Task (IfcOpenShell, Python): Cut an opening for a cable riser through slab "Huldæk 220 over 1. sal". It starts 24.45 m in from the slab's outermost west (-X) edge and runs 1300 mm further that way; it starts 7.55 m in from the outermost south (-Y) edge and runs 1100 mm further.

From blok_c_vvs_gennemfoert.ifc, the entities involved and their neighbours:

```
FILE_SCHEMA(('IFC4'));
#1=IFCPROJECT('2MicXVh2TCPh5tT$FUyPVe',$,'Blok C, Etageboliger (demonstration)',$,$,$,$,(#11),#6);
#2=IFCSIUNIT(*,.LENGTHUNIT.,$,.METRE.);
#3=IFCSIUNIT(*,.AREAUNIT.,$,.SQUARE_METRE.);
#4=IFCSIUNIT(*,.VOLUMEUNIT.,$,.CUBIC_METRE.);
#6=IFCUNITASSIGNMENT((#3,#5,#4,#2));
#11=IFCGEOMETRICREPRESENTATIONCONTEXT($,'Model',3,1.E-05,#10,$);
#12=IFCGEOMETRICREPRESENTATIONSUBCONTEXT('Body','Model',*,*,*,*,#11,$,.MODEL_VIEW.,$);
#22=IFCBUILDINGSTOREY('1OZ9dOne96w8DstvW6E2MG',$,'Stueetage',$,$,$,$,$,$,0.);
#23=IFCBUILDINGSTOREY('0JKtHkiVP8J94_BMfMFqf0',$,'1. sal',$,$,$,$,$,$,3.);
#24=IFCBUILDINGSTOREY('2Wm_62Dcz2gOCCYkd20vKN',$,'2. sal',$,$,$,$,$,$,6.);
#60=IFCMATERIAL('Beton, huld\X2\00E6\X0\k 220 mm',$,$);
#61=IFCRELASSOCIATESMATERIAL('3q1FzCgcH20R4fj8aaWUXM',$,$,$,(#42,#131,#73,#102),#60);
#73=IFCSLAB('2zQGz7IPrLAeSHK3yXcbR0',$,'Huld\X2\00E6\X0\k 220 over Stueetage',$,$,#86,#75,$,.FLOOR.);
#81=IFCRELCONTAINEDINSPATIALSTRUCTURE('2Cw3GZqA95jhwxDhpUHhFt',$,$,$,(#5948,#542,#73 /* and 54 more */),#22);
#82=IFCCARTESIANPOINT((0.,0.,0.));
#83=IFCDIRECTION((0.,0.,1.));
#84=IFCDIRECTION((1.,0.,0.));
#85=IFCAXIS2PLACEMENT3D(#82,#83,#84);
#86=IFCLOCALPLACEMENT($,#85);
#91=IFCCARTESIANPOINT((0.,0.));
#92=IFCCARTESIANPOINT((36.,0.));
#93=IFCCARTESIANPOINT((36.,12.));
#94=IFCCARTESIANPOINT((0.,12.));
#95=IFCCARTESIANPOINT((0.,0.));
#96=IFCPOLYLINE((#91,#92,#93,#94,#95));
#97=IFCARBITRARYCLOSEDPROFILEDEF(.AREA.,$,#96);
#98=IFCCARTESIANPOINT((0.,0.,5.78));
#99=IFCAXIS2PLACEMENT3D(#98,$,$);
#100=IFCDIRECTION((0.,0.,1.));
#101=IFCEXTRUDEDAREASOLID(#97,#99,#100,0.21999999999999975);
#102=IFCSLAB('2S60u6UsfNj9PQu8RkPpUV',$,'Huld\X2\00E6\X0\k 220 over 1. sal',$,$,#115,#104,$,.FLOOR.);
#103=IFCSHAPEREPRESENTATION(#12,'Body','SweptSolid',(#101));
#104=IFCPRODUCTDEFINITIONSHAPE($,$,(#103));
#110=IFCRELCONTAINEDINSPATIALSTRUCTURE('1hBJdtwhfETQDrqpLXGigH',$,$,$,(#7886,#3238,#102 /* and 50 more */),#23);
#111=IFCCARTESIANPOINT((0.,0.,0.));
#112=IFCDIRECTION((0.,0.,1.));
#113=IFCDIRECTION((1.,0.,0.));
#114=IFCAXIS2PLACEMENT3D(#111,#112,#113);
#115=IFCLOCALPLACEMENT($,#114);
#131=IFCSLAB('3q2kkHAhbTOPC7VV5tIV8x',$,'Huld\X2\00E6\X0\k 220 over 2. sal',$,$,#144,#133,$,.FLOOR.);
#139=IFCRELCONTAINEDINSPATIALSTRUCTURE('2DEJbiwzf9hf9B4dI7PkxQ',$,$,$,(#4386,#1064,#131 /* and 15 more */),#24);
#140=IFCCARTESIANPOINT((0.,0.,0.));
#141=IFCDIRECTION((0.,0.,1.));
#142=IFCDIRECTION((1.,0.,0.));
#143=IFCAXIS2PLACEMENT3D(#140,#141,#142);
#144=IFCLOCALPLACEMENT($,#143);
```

```python
import numpy as np
import ifcopenshell
import ifcopenshell.api.feature
import ifcopenshell.api.geometry
import ifcopenshell.api.root
import ifcopenshell.geom
import ifcopenshell.util.placement
import ifcopenshell.util.representation
import ifcopenshell.util.shape
import ifcopenshell.util.unit

model = ifcopenshell.open("blok_c_vvs_gennemfoert.ifc")
unit_scale = ifcopenshell.util.unit.calculate_unit_scale(model)
settings = ifcopenshell.geom.settings()


def volume(element):
    """Net volume in cubic metres, openings subtracted."""
    shape = ifcopenshell.geom.create_shape(settings, element)
    return ifcopenshell.util.shape.get_volume(shape.geometry)


slab = model.by_guid("2S60u6UsfNj9PQu8RkPpUV")
before = volume(slab)

# Extent in the slab's own axes, in metres. The edges named are its -X and -Y sides.
slab_shape = ifcopenshell.geom.create_shape(settings, slab)
vertices = ifcopenshell.util.shape.get_vertices(slab_shape.geometry)
x_min, y_min, bottom = vertices.min(axis=0)
top = vertices[:, 2].max()

opening = ifcopenshell.api.root.create_entity(model, ifc_class="IfcOpeningElement", name="Cable riser opening", predefined_type="OPENING")
context = ifcopenshell.util.representation.get_context(model, "Model", "Body", "MODEL_VIEW")
width, depth = 1.3, 1.1
outline = [(0.0, 0.0), (width, 0.0), (width, depth), (0.0, depth), (0.0, 0.0)]
# Overshoot both faces by 50 mm so the cut is clean.
shape = ifcopenshell.api.geometry.add_slab_representation(
    model, context=context, depth=top - bottom + 0.1, polyline=outline
)
ifcopenshell.api.geometry.assign_representation(model, product=opening, representation=shape)

matrix = ifcopenshell.util.placement.get_local_placement(slab.ObjectPlacement)
matrix[:, 3] = matrix @ np.append(np.array([x_min + 24.45, y_min + 7.55, bottom - 0.05]) / unit_scale, 1.0)
ifcopenshell.api.geometry.edit_object_placement(model, product=opening, matrix=matrix, is_si=False)
ifcopenshell.api.feature.add_feature(model, feature=opening, element=slab)

after = volume(slab)

print(f"slab volume {before:.3f} -> {after:.3f} m3")

model.write("blok_c_vvs_gennemfoert_updated.ifc")
```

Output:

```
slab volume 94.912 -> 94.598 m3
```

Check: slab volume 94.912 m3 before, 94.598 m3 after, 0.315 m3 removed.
